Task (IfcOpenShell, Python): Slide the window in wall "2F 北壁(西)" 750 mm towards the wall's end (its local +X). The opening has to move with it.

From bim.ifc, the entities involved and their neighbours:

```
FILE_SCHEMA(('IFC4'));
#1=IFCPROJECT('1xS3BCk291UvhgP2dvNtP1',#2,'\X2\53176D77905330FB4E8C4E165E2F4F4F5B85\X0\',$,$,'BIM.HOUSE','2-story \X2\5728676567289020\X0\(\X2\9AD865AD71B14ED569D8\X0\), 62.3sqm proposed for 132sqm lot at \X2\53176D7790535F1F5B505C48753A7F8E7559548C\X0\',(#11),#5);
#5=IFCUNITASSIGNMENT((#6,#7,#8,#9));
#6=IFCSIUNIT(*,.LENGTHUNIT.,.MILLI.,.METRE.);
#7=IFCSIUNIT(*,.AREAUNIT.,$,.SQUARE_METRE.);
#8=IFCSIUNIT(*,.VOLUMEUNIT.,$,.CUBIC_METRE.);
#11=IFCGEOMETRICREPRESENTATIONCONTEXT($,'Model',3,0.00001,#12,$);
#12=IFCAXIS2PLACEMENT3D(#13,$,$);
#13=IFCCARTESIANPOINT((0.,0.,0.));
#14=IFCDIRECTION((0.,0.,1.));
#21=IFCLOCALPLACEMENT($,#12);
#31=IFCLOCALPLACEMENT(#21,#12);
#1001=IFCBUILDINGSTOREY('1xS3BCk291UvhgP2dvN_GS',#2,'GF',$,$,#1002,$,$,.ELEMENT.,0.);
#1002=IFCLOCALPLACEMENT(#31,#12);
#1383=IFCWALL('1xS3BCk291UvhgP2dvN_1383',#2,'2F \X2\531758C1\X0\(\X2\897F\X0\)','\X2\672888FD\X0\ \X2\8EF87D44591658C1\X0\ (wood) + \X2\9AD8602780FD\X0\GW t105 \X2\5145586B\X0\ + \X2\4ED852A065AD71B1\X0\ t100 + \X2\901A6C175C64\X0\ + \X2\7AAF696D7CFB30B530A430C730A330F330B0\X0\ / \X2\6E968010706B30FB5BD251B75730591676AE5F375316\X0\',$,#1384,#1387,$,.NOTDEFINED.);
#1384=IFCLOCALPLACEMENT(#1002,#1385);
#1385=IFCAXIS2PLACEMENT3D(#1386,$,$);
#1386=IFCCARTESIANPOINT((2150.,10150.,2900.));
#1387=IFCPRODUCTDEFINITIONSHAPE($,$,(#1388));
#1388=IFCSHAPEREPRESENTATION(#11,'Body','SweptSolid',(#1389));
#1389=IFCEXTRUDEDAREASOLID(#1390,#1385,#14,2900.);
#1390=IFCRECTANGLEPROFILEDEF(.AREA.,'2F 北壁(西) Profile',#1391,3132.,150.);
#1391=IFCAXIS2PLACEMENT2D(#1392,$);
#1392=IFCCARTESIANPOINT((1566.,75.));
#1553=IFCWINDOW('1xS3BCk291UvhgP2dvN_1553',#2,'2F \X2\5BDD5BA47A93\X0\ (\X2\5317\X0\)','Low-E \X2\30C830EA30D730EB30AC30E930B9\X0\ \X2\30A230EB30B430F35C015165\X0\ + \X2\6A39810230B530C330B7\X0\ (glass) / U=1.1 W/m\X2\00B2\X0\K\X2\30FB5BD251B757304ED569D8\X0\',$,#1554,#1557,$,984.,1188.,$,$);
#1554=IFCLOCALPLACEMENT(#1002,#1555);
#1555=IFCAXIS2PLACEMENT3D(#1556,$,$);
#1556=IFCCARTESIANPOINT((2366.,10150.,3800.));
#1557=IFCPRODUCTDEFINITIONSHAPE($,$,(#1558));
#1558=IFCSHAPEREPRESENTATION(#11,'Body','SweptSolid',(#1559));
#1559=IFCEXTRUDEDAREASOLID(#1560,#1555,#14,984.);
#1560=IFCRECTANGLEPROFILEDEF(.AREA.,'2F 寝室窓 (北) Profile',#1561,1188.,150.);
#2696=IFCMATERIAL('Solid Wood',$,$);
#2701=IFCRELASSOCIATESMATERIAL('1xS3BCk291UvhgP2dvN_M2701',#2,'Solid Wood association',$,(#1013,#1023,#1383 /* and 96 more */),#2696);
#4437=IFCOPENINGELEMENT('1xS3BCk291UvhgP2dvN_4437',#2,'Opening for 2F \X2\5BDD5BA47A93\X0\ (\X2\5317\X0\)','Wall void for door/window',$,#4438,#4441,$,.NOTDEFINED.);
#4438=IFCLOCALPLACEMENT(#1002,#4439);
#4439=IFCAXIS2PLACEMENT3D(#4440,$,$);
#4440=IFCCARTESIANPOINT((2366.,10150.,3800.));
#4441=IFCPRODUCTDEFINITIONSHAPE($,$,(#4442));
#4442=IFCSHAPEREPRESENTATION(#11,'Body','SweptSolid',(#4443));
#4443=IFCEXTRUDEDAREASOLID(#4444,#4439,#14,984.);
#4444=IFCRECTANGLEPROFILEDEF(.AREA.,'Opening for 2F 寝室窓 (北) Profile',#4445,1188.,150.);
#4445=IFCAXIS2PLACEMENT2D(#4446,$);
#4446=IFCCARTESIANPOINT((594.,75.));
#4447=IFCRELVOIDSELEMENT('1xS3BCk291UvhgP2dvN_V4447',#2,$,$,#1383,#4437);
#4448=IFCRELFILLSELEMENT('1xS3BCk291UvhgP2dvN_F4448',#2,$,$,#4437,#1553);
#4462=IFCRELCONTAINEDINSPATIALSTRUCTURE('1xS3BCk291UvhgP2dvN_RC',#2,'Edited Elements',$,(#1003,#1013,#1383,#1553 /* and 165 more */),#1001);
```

```python
import ifcopenshell
import ifcopenshell.api.geometry
import ifcopenshell.util.placement
import ifcopenshell.util.unit

model = ifcopenshell.open("bim.ifc")
unit_scale = ifcopenshell.util.unit.calculate_unit_scale(model)

window = model.by_guid("1xS3BCk291UvhgP2dvN_1553")
opening = window.FillsVoids[0].RelatingOpeningElement
wall = opening.VoidsElements[0].RelatingBuildingElement

wall_matrix = ifcopenshell.util.placement.get_local_placement(wall.ObjectPlacement)
shift = wall_matrix[:3, 0] * 0.75 / unit_scale
before = ifcopenshell.util.placement.get_local_placement(window.ObjectPlacement)[:3, 3].copy()

# The window is not placed relative to its opening, so move both.
for product in (opening, window):
    matrix = ifcopenshell.util.placement.get_local_placement(product.ObjectPlacement)
    matrix[:3, 3] += shift
    ifcopenshell.api.geometry.edit_object_placement(model, product=product, matrix=matrix, is_si=False)

after = ifcopenshell.util.placement.get_local_placement(window.ObjectPlacement)[:3, 3]
print("window moved by", (after - before).round(3) + 0.0)

model.write("bim-out.ifc")
```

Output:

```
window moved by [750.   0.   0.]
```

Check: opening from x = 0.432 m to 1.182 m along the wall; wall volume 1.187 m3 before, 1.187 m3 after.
